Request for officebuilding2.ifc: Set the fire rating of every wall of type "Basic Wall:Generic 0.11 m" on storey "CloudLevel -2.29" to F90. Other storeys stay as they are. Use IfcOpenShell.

First a look at what the model holds.

```python
import ifcopenshell
import ifcopenshell.util.element

model = ifcopenshell.open("officebuilding2.ifc")
print(model.schema)
storey = next(s for s in model.by_type("IfcBuildingStorey") if s.Name == "CloudLevel -2.29")
walls = [e for e in ifcopenshell.util.element.get_decomposition(storey) if e.is_a("IfcWall")]
seen = {}
for e in walls:
    element_type = ifcopenshell.util.element.get_type(e)
    key = (element_type.Name if element_type != e and element_type else None, ifcopenshell.util.element.get_pset(e, "Pset_WallCommon", "FireRating"))
    seen[key] = seen.get(key, 0) + 1
for (name, value), count in sorted(seen.items(), key=str):
    print(count, "x", name, "|", value)
```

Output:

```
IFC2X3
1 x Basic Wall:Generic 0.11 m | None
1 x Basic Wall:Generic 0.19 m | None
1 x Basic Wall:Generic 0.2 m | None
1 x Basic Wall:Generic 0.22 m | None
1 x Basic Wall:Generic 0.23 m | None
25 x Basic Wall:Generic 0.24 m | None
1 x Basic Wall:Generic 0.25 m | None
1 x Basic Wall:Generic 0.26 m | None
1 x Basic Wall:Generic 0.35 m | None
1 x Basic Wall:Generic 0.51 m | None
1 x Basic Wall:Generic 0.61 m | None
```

```python
import ifcopenshell
import ifcopenshell.api.pset
import ifcopenshell.util.element

model = ifcopenshell.open("officebuilding2.ifc")

storey = next(s for s in model.by_type("IfcBuildingStorey") if s.Name == "CloudLevel -2.29")
walls = [e for e in ifcopenshell.util.element.get_decomposition(storey) if e.is_a("IfcWall")]

count = 0
for e in walls:
    element_type = ifcopenshell.util.element.get_type(e)
    if element_type in (None, e) or element_type.Name != "Basic Wall:Generic 0.11 m":
        continue
    # add_pset returns the element's existing set when there is one.
    pset = ifcopenshell.api.pset.add_pset(model, product=e, name="Pset_WallCommon")
    ifcopenshell.api.pset.edit_pset(model, pset=pset, properties={"FireRating": "F90"})
    count += 1

print(count, "walls updated")

model.write("officebuilding2-out.ifc")
```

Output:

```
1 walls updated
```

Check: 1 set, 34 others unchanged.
